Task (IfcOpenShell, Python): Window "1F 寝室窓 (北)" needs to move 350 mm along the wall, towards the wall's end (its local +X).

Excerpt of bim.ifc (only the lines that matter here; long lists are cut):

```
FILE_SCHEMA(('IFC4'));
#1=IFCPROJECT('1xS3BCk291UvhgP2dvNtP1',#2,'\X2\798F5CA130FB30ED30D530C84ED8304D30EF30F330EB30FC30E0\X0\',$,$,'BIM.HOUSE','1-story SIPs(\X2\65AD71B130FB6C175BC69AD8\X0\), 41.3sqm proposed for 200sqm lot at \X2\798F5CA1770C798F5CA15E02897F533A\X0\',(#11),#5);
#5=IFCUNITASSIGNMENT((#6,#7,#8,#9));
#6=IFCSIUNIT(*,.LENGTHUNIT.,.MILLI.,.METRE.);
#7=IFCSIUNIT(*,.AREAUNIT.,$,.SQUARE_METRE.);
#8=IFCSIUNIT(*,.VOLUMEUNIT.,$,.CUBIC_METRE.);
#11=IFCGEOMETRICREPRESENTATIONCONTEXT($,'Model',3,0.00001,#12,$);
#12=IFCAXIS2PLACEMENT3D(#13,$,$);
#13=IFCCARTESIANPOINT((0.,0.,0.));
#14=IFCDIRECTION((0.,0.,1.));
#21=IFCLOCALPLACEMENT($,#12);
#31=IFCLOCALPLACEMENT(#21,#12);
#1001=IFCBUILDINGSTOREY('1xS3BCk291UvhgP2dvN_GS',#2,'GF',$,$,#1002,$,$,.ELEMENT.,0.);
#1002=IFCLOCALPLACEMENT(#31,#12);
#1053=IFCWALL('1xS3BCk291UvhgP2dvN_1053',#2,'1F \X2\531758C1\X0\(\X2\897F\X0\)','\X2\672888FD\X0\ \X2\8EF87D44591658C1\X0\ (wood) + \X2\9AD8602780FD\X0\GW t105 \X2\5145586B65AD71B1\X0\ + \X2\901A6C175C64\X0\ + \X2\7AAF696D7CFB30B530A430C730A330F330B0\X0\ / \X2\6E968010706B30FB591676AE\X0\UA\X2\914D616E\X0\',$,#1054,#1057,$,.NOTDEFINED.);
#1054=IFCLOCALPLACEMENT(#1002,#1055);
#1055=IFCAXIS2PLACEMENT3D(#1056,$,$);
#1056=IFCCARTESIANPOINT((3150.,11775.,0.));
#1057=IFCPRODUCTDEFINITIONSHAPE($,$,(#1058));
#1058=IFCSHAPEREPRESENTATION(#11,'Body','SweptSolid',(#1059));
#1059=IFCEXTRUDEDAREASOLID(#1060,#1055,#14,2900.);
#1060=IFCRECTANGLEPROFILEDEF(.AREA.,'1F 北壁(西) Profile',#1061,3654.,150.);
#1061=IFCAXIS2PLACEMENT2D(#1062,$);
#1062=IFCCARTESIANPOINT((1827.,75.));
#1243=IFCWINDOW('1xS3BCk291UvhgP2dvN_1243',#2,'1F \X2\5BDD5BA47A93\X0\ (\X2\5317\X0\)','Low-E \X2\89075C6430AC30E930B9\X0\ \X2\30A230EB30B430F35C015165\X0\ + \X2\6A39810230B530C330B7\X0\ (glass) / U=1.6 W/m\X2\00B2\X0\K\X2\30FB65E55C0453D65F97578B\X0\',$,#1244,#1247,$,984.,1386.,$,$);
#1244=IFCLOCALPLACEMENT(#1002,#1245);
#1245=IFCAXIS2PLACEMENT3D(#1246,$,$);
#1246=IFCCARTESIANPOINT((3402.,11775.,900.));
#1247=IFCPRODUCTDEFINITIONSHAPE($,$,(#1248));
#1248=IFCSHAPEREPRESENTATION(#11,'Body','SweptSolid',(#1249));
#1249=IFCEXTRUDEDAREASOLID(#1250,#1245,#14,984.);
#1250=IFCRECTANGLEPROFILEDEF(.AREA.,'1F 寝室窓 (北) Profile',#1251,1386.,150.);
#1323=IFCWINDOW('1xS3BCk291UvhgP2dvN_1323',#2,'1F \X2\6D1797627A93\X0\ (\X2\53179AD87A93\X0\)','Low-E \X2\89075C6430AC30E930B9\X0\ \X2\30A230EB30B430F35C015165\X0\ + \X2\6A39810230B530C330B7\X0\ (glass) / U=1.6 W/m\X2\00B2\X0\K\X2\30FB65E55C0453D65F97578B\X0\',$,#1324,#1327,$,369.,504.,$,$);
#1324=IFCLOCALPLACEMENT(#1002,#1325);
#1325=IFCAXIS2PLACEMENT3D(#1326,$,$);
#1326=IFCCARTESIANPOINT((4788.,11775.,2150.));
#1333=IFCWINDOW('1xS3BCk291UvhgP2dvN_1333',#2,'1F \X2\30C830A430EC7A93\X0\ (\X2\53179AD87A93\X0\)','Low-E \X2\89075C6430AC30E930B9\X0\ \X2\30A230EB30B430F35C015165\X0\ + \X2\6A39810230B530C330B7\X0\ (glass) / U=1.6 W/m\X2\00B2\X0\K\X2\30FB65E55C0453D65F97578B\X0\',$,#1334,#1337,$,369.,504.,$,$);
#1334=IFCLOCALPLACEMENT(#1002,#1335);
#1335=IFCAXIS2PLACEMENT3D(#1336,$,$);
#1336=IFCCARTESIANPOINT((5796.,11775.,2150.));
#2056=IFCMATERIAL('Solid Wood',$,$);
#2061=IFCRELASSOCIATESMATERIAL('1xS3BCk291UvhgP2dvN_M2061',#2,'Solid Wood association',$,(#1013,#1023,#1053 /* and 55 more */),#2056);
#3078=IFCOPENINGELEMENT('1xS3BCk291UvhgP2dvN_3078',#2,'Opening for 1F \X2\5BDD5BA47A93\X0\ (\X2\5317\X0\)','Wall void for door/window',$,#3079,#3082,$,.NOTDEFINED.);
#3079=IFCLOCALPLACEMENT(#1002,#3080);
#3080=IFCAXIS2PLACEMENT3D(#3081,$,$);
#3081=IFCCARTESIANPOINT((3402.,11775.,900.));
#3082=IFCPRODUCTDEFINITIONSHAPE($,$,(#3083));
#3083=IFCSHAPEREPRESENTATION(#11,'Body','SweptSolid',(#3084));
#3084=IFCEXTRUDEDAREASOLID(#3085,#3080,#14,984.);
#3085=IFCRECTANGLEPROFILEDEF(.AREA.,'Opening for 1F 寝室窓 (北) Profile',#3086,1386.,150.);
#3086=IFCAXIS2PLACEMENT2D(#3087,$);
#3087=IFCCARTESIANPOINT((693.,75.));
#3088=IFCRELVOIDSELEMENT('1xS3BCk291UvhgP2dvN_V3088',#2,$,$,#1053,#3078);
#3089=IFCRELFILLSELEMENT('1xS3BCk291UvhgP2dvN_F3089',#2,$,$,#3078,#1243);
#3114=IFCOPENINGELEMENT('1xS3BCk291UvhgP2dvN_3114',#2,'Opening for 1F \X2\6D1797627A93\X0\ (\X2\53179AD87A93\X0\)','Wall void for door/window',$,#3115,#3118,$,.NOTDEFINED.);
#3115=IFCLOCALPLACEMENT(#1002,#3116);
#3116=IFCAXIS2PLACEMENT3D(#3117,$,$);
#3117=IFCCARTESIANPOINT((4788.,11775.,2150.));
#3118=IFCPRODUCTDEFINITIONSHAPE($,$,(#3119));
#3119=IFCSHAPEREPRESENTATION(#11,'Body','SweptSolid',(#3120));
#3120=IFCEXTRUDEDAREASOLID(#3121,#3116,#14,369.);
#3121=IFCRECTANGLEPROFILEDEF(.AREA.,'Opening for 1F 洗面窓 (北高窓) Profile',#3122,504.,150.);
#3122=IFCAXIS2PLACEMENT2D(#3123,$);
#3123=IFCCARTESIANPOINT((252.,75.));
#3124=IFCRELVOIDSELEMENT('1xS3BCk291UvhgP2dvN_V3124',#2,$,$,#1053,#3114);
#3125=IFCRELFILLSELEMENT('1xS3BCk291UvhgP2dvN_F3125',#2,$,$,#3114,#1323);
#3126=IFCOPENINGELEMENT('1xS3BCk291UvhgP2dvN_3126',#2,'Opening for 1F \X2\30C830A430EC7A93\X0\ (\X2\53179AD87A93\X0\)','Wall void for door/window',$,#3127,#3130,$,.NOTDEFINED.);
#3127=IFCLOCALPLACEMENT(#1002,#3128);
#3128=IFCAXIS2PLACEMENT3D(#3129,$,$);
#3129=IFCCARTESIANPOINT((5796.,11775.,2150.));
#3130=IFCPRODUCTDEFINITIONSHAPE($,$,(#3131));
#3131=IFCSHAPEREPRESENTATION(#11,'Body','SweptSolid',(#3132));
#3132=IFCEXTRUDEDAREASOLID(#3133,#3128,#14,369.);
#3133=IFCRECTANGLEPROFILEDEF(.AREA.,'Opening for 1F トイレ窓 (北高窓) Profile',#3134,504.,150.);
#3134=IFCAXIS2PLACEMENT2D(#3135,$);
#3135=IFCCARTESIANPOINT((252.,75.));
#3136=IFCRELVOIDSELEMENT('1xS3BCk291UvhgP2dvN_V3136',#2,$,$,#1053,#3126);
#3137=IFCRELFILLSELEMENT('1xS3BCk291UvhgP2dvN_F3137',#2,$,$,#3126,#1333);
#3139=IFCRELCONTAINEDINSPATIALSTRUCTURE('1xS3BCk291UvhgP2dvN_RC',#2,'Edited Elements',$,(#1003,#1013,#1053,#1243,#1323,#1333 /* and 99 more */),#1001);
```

```python
import ifcopenshell
import ifcopenshell.api.geometry
import ifcopenshell.util.placement

model = ifcopenshell.open("bim.ifc")

window = model.by_guid("1xS3BCk291UvhgP2dvN_1243")
opening = window.FillsVoids[0].RelatingOpeningElement
wall = opening.VoidsElements[0].RelatingBuildingElement

wall_matrix = ifcopenshell.util.placement.get_local_placement(wall.ObjectPlacement)
shift = wall_matrix[:3, 0] * 350.0
before = ifcopenshell.util.placement.get_local_placement(window.ObjectPlacement)[:3, 3].copy()

# The window is not placed relative to its opening, so move both.
for product in (opening, window):
    matrix = ifcopenshell.util.placement.get_local_placement(product.ObjectPlacement)
    matrix[:3, 3] += shift
    ifcopenshell.api.geometry.edit_object_placement(model, product=product, matrix=matrix, is_si=False)

after = ifcopenshell.util.placement.get_local_placement(window.ObjectPlacement)[:3, 3]
print("window moved by", (after - before).round(3) + 0.0)

model.write("bim_updated.ifc")
```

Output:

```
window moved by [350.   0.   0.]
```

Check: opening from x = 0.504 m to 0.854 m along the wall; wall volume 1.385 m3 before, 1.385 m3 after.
